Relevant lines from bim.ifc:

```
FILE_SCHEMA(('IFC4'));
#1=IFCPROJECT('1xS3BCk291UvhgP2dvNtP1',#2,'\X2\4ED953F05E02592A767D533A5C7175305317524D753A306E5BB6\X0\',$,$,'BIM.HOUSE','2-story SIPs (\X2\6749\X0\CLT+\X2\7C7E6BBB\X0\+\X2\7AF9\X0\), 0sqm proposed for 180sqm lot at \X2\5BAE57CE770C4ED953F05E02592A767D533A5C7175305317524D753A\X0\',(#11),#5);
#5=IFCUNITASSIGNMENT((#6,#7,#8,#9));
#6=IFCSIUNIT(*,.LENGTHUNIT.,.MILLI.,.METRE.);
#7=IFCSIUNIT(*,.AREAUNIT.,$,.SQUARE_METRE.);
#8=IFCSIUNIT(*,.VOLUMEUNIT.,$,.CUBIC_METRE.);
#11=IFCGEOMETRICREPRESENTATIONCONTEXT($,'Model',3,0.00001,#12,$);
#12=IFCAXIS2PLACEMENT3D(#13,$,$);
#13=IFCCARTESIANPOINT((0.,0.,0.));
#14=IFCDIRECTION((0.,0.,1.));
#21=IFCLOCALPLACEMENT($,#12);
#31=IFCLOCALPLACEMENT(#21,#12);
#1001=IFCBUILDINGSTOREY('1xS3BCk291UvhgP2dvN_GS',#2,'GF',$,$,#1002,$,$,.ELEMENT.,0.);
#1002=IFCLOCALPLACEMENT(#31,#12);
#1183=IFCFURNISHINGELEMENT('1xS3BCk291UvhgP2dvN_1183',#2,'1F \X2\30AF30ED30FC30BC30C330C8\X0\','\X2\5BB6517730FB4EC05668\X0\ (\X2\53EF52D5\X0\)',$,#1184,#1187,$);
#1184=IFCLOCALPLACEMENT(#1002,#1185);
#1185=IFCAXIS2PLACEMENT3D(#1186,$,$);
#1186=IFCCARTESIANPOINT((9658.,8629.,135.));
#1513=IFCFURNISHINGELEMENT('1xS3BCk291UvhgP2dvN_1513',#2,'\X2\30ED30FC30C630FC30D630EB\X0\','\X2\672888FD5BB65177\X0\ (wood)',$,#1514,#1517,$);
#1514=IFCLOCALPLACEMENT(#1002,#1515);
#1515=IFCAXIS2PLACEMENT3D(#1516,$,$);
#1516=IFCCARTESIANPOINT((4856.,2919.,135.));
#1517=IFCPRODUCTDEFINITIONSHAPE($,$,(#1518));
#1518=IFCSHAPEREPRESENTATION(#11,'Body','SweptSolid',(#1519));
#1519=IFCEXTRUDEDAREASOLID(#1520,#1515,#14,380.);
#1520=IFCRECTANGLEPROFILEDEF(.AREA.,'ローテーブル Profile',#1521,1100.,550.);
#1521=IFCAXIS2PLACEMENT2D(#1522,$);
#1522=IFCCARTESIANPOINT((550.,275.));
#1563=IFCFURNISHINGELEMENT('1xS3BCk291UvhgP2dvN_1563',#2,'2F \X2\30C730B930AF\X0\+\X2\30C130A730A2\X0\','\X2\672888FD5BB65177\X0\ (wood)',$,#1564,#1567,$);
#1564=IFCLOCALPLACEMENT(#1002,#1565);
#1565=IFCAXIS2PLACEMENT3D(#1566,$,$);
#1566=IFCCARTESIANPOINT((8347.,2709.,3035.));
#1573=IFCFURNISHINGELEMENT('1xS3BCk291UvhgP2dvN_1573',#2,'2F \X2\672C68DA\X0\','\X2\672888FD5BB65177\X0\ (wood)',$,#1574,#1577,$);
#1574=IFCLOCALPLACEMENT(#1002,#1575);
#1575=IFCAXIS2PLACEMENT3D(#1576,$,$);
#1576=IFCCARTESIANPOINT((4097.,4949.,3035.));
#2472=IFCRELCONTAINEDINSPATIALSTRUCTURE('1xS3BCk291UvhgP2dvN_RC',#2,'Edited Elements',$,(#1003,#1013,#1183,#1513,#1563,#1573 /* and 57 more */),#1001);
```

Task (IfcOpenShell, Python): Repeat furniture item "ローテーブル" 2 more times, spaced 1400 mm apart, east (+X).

```python
import numpy as np
import ifcopenshell
import ifcopenshell.api.geometry
import ifcopenshell.api.root
import ifcopenshell.util.element
import ifcopenshell.util.placement

model = ifcopenshell.open("bim.ifc")


def reuse_history(source, copy):
    """copy_class also copies each property set's owner history, people and application; keep the originals."""
    for rel in copy.IsDefinedBy:
        if rel.is_a("IfcRelDefinesByProperties") and (history := rel.RelatingPropertyDefinition.OwnerHistory):
            rel.RelatingPropertyDefinition.OwnerHistory = source.OwnerHistory
            ifcopenshell.util.element.remove_deep2(model, history)


source = model.by_guid("1xS3BCk291UvhgP2dvN_1513")
base = ifcopenshell.util.placement.get_local_placement(source.ObjectPlacement)
step = np.array([1.0, 0.0, 0.0]) * 1400.0

for i in range(1, 3):
    copy = ifcopenshell.api.root.copy_class(model, product=source)
    copy.Representation = ifcopenshell.util.element.copy_deep(
        model, source.Representation, exclude=["IfcGeometricRepresentationContext", "IfcRepresentationMap"]
    )
    reuse_history(source, copy)
    matrix = base.copy()
    matrix[:3, 3] += i * step
    print("added at", matrix[:3, 3].round(3) + 0.0)
    ifcopenshell.api.geometry.edit_object_placement(model, product=copy, matrix=matrix, is_si=False)

model.write("bim-out.ifc")
```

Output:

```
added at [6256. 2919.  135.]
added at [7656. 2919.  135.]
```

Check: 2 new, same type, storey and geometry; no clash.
